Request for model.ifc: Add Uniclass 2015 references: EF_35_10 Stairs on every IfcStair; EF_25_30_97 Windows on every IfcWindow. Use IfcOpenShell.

First a look at what the model holds.

```python
import ifcopenshell

model = ifcopenshell.open("model.ifc")
print(model.schema)
print("classifications:", [c.Name for c in model.by_type("IfcClassification")])
for ifc_class in ("IfcDoor", "IfcRoof", "IfcStair", "IfcWall", "IfcWindow"):
    print(ifc_class, len(model.by_type(ifc_class)))
```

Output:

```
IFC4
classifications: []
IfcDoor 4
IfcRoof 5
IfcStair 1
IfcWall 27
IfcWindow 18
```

```python
import ifcopenshell
import ifcopenshell.api.classification

model = ifcopenshell.open("model.ifc")

system = ifcopenshell.api.classification.add_classification(model, classification="Uniclass 2015")

codes = {
    "IfcStair": ("EF_35_10", "Stairs"),
    "IfcWindow": ("EF_25_30_97", "Windows"),
}
for ifc_class, (code, name) in codes.items():
    products = model.by_type(ifc_class)
    ifcopenshell.api.classification.add_reference(
        model, products=products, classification=system, identification=code, name=name
    )
    print(code, len(products))

model.write("model_v2.ifc")
```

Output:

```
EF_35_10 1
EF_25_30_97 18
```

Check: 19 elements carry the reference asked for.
